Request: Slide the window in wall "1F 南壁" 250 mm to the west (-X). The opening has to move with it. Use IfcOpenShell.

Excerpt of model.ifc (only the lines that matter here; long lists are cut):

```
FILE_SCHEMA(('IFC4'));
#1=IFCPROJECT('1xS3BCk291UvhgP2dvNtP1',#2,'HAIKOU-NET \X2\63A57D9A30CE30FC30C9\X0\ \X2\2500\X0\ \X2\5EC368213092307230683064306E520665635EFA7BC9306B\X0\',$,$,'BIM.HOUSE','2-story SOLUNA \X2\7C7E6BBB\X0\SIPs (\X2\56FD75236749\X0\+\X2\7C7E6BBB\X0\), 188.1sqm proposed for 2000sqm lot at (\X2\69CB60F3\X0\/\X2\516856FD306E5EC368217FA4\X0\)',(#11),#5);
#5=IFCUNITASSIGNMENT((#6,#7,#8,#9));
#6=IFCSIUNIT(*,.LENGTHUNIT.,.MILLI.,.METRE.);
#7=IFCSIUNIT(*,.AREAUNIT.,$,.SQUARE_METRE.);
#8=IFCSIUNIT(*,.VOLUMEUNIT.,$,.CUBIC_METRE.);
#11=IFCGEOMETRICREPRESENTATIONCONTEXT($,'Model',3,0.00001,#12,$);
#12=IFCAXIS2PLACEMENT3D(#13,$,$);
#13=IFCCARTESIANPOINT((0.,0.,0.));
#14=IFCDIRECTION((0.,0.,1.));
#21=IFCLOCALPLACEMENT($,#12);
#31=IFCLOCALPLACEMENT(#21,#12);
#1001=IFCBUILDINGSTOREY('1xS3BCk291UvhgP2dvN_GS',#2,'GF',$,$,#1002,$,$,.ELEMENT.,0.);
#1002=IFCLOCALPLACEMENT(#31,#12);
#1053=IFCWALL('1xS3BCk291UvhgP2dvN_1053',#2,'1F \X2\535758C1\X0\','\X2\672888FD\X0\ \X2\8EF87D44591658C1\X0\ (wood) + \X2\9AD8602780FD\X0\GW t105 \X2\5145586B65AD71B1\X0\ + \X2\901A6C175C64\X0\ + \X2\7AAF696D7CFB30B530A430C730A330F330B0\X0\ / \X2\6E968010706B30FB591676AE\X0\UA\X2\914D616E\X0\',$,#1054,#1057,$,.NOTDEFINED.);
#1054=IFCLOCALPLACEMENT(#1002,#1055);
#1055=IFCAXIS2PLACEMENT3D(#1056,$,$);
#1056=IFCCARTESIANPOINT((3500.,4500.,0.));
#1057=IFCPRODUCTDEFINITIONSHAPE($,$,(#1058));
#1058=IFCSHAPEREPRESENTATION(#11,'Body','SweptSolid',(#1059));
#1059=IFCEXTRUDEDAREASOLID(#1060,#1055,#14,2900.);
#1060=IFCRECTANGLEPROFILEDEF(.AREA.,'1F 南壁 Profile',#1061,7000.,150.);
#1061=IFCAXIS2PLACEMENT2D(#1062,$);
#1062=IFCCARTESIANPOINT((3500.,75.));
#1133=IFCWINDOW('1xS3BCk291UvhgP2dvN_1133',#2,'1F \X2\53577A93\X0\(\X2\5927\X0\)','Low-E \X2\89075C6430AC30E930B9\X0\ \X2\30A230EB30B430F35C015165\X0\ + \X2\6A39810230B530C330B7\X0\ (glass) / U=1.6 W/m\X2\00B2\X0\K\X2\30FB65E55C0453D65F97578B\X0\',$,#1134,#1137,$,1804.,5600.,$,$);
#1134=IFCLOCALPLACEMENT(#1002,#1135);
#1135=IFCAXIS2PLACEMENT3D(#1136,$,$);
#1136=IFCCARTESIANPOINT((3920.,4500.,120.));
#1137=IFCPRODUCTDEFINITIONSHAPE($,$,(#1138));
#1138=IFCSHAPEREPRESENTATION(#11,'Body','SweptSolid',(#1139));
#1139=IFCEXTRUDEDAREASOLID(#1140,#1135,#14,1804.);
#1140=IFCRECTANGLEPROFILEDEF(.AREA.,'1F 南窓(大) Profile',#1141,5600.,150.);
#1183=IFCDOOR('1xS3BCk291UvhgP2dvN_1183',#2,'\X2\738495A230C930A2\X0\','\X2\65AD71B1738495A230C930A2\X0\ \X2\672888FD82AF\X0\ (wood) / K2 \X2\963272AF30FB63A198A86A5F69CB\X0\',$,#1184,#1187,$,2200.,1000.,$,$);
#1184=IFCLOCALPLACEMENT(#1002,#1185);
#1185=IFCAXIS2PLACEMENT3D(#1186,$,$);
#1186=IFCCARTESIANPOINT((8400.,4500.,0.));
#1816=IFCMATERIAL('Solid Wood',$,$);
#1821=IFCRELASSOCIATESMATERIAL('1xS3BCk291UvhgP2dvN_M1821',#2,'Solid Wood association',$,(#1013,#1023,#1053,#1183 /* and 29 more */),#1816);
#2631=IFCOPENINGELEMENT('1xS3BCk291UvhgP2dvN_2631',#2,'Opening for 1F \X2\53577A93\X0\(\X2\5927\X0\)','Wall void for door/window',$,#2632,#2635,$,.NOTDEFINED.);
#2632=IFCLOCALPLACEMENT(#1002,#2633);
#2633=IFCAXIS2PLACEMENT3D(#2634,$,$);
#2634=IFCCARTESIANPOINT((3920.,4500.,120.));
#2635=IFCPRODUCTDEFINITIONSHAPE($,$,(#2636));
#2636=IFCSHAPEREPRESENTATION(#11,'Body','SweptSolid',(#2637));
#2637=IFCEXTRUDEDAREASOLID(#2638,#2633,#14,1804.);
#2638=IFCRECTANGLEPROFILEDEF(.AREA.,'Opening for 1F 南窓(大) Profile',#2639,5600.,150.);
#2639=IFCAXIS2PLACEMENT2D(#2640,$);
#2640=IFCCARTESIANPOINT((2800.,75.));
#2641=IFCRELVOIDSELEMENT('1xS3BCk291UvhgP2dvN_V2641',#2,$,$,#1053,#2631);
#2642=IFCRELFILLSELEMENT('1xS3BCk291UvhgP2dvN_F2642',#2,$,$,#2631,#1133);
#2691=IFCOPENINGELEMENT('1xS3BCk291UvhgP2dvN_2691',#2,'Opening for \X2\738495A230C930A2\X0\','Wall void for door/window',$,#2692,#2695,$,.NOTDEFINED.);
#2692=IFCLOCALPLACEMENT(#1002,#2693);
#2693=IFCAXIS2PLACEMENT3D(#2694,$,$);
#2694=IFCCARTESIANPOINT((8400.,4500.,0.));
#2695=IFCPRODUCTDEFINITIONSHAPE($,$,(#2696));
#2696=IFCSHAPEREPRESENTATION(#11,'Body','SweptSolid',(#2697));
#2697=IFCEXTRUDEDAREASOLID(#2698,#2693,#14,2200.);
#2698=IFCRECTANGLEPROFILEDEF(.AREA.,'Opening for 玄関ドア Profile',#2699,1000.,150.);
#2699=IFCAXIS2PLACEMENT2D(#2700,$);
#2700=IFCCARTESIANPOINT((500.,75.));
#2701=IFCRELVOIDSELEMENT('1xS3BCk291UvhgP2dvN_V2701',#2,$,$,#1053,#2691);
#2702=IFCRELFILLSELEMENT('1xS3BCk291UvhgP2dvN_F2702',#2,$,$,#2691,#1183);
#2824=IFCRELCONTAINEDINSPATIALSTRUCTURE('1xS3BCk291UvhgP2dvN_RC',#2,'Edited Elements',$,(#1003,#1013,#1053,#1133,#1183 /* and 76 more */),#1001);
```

```python
import ifcopenshell
import ifcopenshell.api.geometry
import ifcopenshell.util.placement
import ifcopenshell.util.unit

model = ifcopenshell.open("model.ifc")
unit_scale = ifcopenshell.util.unit.calculate_unit_scale(model)

window = model.by_id(1133)
opening = window.FillsVoids[0].RelatingOpeningElement
wall = opening.VoidsElements[0].RelatingBuildingElement

wall_matrix = ifcopenshell.util.placement.get_local_placement(wall.ObjectPlacement)
shift = wall_matrix[:3, 0] * -0.25 / unit_scale
before = ifcopenshell.util.placement.get_local_placement(window.ObjectPlacement)[:3, 3].copy()

# The window is not placed relative to its opening, so move both.
for product in (opening, window):
    matrix = ifcopenshell.util.placement.get_local_placement(product.ObjectPlacement)
    matrix[:3, 3] += shift
    ifcopenshell.api.geometry.edit_object_placement(model, product=product, matrix=matrix, is_si=False)

after = ifcopenshell.util.placement.get_local_placement(window.ObjectPlacement)[:3, 3]
print("window moved by", (after - before).round(3) + 0.0)

model.write("model-out.ifc")
```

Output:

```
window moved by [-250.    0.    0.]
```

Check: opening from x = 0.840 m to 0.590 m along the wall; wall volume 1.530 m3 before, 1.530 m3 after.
